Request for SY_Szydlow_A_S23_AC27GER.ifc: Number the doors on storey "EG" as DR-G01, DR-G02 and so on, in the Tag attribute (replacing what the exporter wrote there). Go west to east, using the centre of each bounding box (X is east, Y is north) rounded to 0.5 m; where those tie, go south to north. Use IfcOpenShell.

First a look at what the model holds.

```python
import ifcopenshell
import ifcopenshell.util.element
import ifcopenshell.util.placement

model = ifcopenshell.open("SY_Szydlow_A_S23_AC27GER.ifc")
print(model.schema)
storey = next(s for s in model.by_type("IfcBuildingStorey") if s.Name == "EG")
doors = [e for e in ifcopenshell.util.element.get_decomposition(storey) if e.is_a("IfcDoor")]
for e in sorted(doors, key=lambda e: e.id()):
    origin = ifcopenshell.util.placement.get_local_placement(e.ObjectPlacement)[:3, 3]
    print(e.id(), e.Tag, e.Name, origin.round(2) + 0.0, sep=" | ")
```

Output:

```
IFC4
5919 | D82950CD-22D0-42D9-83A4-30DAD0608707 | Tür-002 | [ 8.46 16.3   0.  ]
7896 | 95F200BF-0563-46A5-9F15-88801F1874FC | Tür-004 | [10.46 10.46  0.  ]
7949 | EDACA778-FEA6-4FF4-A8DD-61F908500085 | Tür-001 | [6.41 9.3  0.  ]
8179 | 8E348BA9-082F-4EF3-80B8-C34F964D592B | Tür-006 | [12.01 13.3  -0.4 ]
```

```python
import ifcopenshell
import ifcopenshell.geom
import ifcopenshell.util.element
import ifcopenshell.util.shape

model = ifcopenshell.open("SY_Szydlow_A_S23_AC27GER.ifc")
settings = ifcopenshell.geom.settings()
settings.set("use-world-coords", True)


def centre(element):
    shape = ifcopenshell.geom.create_shape(settings, element)
    return ifcopenshell.util.shape.get_bbox_centroid(shape.geometry)


storey = next(s for s in model.by_type("IfcBuildingStorey") if s.Name == "EG")
doors = [e for e in ifcopenshell.util.element.get_decomposition(storey) if e.is_a("IfcDoor")]

# Insertion points can sit at a corner or the storey origin, so sort by the geometry (in metres).
centres = {e: centre(e) for e in doors}
doors.sort(key=lambda e: (round(centres[e][0] / 0.5), centres[e][1]))

for i, e in enumerate(doors, start=1):
    number = f"DR-G{i:02d}"
    e.Tag = number
    print(e.id(), number)

model.write("SY_Szydlow_A_S23_AC27GER_updated.ifc")
```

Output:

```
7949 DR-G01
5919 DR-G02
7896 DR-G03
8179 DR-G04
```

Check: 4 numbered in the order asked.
